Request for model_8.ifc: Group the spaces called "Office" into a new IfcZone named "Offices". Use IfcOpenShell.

First a look at what the model holds.

```python
import ifcopenshell

model = ifcopenshell.open("model_8.ifc")
print(model.schema)
seen = {}
for space in model.by_type("IfcSpace"):
    seen[space.LongName] = seen.get(space.LongName, 0) + 1
for name, count in sorted(seen.items(), key=str):
    print(count, "x", name)
print("zones:", [z.Name for z in model.by_type("IfcZone")][:20])
```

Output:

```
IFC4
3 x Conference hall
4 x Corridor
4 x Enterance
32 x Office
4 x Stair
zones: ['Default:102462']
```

```python
import ifcopenshell
import ifcopenshell.api.group
import ifcopenshell.api.root

model = ifcopenshell.open("model_8.ifc")

names = {"Office"}
spaces = [s for s in model.by_type("IfcSpace") if s.LongName in names]

zone = ifcopenshell.api.root.create_entity(model, ifc_class="IfcZone", name="Offices")
ifcopenshell.api.group.assign_group(model, products=spaces, group=zone)
print(len(spaces), "spaces in", zone.Name)

model.write("model_8-out.ifc")
```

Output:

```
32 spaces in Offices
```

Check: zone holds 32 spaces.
